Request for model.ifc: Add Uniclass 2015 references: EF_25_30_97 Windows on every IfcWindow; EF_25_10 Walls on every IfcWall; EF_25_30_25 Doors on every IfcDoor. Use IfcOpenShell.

First a look at what the model holds.

```python
import ifcopenshell

model = ifcopenshell.open("model.ifc")
print(model.schema)
print("classifications:", [c.Name for c in model.by_type("IfcClassification")])
for ifc_class in ("IfcDoor", "IfcRoof", "IfcStair", "IfcWall", "IfcWindow"):
    print(ifc_class, len(model.by_type(ifc_class)))
```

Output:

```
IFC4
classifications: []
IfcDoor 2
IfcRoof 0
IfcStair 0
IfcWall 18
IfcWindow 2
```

```python
import ifcopenshell
import ifcopenshell.api.classification

model = ifcopenshell.open("model.ifc")

system = ifcopenshell.api.classification.add_classification(model, classification="Uniclass 2015")

codes = {
    "IfcWindow": ("EF_25_30_97", "Windows"),
    "IfcWall": ("EF_25_10", "Walls"),
    "IfcDoor": ("EF_25_30_25", "Doors"),
}
for ifc_class, (code, name) in codes.items():
    products = model.by_type(ifc_class)
    ifcopenshell.api.classification.add_reference(
        model, products=products, classification=system, identification=code, name=name
    )
    print(code, len(products))

model.write("model_rev.ifc")
```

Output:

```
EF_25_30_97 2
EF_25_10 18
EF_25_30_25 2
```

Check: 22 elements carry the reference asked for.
